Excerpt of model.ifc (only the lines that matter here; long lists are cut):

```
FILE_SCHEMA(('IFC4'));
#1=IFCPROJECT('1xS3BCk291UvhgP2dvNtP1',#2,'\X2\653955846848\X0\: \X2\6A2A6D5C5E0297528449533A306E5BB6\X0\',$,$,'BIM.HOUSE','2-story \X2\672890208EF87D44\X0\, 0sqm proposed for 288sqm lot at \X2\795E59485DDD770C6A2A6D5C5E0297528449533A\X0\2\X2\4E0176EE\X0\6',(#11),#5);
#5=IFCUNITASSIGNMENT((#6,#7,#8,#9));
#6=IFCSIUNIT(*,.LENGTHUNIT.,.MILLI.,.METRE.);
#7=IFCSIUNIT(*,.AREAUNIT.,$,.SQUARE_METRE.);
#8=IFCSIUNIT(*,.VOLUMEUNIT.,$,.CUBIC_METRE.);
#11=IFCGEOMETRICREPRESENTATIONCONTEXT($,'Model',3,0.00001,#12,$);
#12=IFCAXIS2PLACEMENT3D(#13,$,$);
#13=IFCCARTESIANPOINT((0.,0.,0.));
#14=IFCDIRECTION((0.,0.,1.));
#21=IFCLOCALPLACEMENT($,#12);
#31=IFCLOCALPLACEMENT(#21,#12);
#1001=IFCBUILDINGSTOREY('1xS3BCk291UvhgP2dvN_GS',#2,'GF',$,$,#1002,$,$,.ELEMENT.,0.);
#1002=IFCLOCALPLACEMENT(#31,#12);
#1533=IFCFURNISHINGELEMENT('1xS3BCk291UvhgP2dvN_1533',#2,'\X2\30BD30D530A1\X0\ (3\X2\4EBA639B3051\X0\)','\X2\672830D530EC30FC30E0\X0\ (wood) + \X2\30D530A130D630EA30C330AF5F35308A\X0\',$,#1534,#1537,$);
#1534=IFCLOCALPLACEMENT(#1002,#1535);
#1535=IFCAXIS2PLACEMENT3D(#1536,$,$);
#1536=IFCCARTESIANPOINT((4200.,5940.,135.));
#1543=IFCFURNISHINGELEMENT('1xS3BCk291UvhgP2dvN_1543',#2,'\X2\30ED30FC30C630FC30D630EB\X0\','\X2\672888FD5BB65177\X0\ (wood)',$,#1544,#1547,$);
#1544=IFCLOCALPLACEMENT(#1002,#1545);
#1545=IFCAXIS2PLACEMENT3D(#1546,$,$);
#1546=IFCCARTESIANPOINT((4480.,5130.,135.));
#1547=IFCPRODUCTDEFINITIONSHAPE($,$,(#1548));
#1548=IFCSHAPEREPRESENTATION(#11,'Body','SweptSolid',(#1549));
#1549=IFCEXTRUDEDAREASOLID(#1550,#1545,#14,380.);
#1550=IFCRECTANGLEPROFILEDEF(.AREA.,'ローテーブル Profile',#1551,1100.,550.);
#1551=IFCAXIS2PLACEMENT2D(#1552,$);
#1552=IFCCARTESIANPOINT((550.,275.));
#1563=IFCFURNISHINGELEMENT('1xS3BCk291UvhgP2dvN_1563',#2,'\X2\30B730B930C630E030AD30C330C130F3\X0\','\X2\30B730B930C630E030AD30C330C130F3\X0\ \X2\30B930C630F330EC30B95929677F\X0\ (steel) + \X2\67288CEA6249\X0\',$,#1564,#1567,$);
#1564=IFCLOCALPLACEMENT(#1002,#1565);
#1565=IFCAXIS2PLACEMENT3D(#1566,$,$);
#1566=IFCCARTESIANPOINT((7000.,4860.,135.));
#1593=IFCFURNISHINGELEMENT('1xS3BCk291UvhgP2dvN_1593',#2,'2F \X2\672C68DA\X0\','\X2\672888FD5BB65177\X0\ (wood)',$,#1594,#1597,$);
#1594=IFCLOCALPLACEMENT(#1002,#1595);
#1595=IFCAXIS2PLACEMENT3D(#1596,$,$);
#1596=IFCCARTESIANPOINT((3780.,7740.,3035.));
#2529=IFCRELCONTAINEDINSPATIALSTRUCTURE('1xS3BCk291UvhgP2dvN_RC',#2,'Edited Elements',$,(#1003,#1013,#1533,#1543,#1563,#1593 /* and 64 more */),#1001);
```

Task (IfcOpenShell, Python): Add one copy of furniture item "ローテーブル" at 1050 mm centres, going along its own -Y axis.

```python
import ifcopenshell
import ifcopenshell.api.geometry
import ifcopenshell.api.root
import ifcopenshell.util.element
import ifcopenshell.util.placement
import ifcopenshell.util.unit

model = ifcopenshell.open("model.ifc")
unit_scale = ifcopenshell.util.unit.calculate_unit_scale(model)


def reuse_history(source, copy):
    """copy_class also copies each property set's owner history, people and application; keep the originals."""
    for rel in copy.IsDefinedBy:
        if rel.is_a("IfcRelDefinesByProperties") and (history := rel.RelatingPropertyDefinition.OwnerHistory):
            rel.RelatingPropertyDefinition.OwnerHistory = source.OwnerHistory
            ifcopenshell.util.element.remove_deep2(model, history)


source = model.by_id(1543)
base = ifcopenshell.util.placement.get_local_placement(source.ObjectPlacement)
step = -base[:3, 1] * 1.05 / unit_scale

for i in range(1, 2):
    copy = ifcopenshell.api.root.copy_class(model, product=source)
    copy.Representation = ifcopenshell.util.element.copy_deep(
        model, source.Representation, exclude=["IfcGeometricRepresentationContext", "IfcRepresentationMap"]
    )
    reuse_history(source, copy)
    matrix = base.copy()
    matrix[:3, 3] += i * step
    print("added at", matrix[:3, 3].round(3) + 0.0)
    ifcopenshell.api.geometry.edit_object_placement(model, product=copy, matrix=matrix, is_si=False)

model.write("model-out.ifc")
```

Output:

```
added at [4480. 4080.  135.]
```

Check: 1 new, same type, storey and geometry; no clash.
